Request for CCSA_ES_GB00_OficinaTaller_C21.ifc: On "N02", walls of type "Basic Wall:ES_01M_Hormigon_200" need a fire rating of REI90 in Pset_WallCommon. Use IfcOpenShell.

First a look at what the model holds.

```python
import ifcopenshell
import ifcopenshell.util.element

model = ifcopenshell.open("CCSA_ES_GB00_OficinaTaller_C21.ifc")
print(model.schema)
storey = next(s for s in model.by_type("IfcBuildingStorey") if s.Name == "N02")
walls = [e for e in ifcopenshell.util.element.get_decomposition(storey) if e.is_a("IfcWall")]
seen = {}
for e in walls:
    element_type = ifcopenshell.util.element.get_type(e)
    key = (element_type.Name if element_type != e and element_type else None, ifcopenshell.util.element.get_pset(e, "Pset_WallCommon", "FireRating"))
    seen[key] = seen.get(key, 0) + 1
for (name, value), count in sorted(seen.items(), key=str):
    print(count, "x", name, "|", value)
```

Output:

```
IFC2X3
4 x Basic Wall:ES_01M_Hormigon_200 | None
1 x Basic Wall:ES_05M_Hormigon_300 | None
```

```python
import ifcopenshell
import ifcopenshell.api.pset
import ifcopenshell.util.element

model = ifcopenshell.open("CCSA_ES_GB00_OficinaTaller_C21.ifc")

storey = next(s for s in model.by_type("IfcBuildingStorey") if s.Name == "N02")
walls = [e for e in ifcopenshell.util.element.get_decomposition(storey) if e.is_a("IfcWall")]

count = 0
for e in walls:
    element_type = ifcopenshell.util.element.get_type(e)
    if element_type in (None, e) or element_type.Name != "Basic Wall:ES_01M_Hormigon_200":
        continue
    # add_pset returns the element's existing set when there is one.
    pset = ifcopenshell.api.pset.add_pset(model, product=e, name="Pset_WallCommon")
    ifcopenshell.api.pset.edit_pset(model, pset=pset, properties={"FireRating": "REI90"})
    count += 1

print(count, "walls updated")

model.write("CCSA_ES_GB00_OficinaTaller_C21_v2.ifc")
```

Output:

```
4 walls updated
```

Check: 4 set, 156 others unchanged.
